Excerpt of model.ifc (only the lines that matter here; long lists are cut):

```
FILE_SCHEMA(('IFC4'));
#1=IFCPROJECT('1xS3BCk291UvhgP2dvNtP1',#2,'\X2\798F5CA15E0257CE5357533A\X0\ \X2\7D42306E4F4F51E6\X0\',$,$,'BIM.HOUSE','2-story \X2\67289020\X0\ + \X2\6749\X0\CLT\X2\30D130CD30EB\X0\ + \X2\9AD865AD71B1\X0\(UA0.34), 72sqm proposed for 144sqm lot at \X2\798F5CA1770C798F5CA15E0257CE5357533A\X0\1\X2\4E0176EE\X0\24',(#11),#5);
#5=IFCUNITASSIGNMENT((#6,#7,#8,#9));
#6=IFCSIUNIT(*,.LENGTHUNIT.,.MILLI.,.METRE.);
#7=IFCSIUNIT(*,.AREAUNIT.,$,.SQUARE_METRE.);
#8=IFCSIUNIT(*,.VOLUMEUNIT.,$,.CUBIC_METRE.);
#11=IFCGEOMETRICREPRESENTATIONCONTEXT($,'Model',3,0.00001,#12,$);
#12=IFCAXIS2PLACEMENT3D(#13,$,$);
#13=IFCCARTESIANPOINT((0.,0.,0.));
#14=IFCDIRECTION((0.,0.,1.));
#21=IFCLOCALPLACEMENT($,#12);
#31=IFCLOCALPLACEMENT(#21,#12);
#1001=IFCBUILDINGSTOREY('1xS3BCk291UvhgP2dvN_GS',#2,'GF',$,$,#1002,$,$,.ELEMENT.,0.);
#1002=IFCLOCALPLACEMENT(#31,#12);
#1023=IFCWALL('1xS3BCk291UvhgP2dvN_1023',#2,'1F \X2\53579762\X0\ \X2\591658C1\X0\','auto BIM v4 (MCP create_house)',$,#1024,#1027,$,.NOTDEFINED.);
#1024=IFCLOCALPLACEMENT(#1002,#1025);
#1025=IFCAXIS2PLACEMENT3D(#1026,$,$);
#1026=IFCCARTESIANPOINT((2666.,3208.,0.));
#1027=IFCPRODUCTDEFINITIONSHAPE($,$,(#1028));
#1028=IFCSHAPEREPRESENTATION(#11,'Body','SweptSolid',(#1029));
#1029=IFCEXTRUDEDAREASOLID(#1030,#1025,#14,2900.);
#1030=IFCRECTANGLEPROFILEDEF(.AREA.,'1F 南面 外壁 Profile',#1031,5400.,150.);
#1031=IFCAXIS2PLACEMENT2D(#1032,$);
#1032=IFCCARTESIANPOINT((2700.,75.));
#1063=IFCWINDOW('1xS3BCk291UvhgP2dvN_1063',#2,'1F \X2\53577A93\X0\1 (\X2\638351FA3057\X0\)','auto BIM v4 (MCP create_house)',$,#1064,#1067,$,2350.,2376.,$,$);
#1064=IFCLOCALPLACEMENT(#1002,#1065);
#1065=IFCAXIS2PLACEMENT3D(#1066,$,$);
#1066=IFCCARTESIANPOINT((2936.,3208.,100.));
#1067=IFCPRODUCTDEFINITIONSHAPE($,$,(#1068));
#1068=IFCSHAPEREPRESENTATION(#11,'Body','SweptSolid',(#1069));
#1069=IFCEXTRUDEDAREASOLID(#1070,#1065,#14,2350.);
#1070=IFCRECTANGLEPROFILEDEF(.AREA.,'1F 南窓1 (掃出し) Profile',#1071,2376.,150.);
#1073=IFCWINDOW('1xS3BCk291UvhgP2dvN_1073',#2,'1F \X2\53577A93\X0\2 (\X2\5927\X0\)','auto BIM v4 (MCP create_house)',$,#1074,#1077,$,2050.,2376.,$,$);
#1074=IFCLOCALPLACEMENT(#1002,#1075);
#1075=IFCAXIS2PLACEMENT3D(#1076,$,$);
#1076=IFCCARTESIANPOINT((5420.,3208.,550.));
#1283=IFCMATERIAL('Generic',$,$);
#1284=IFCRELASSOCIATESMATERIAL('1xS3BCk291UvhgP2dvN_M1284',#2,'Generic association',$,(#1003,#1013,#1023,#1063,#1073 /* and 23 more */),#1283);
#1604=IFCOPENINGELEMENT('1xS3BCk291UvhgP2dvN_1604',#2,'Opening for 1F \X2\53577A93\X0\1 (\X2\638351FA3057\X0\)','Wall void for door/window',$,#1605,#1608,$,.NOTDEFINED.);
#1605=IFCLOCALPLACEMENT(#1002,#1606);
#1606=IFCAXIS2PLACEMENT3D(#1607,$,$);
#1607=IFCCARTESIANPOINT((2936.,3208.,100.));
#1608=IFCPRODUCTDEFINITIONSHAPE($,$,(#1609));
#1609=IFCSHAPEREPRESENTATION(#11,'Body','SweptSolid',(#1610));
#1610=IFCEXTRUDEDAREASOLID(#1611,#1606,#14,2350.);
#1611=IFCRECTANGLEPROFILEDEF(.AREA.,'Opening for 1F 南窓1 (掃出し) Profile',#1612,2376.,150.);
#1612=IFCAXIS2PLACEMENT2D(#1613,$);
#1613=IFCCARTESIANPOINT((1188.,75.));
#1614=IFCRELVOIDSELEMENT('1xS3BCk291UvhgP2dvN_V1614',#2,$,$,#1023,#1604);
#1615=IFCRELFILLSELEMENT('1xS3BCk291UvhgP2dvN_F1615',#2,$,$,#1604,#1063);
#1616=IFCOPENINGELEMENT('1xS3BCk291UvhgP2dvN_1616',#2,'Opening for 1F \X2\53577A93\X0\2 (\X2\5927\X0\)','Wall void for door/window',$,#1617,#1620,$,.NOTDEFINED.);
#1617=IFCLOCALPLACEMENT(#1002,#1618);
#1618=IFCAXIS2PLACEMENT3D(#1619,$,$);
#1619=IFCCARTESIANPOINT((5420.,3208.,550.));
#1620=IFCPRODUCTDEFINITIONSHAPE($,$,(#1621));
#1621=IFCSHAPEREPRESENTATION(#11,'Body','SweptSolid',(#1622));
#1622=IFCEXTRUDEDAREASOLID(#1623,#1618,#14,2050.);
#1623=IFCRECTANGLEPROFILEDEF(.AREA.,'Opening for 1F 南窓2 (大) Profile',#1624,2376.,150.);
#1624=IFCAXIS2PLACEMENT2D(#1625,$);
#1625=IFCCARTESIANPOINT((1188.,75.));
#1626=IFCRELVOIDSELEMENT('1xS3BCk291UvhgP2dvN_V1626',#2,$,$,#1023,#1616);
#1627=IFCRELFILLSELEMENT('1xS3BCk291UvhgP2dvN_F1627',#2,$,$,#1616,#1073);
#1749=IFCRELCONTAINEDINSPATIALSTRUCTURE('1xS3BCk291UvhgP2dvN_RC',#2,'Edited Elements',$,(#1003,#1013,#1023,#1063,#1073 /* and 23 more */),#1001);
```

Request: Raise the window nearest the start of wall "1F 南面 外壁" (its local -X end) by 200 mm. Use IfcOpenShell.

```python
import numpy as np
import ifcopenshell
import ifcopenshell.api.geometry
import ifcopenshell.util.placement
import ifcopenshell.util.unit

model = ifcopenshell.open("model.ifc")
unit_scale = ifcopenshell.util.unit.calculate_unit_scale(model)

window = model.by_id(1063)
opening = window.FillsVoids[0].RelatingOpeningElement
dz = 0.2 / unit_scale

shift = np.array([0.0, 0.0, dz])
# The window is not placed relative to its opening, so move both.
for product in (opening, window):
    matrix = ifcopenshell.util.placement.get_local_placement(product.ObjectPlacement)
    matrix[:3, 3] += shift
    ifcopenshell.api.geometry.edit_object_placement(model, product=product, matrix=matrix, is_si=False)

print(f"moved by {dz * unit_scale:+.3f} m")

model.write("model_updated.ifc")
```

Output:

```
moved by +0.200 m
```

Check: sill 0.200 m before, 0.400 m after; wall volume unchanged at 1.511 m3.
